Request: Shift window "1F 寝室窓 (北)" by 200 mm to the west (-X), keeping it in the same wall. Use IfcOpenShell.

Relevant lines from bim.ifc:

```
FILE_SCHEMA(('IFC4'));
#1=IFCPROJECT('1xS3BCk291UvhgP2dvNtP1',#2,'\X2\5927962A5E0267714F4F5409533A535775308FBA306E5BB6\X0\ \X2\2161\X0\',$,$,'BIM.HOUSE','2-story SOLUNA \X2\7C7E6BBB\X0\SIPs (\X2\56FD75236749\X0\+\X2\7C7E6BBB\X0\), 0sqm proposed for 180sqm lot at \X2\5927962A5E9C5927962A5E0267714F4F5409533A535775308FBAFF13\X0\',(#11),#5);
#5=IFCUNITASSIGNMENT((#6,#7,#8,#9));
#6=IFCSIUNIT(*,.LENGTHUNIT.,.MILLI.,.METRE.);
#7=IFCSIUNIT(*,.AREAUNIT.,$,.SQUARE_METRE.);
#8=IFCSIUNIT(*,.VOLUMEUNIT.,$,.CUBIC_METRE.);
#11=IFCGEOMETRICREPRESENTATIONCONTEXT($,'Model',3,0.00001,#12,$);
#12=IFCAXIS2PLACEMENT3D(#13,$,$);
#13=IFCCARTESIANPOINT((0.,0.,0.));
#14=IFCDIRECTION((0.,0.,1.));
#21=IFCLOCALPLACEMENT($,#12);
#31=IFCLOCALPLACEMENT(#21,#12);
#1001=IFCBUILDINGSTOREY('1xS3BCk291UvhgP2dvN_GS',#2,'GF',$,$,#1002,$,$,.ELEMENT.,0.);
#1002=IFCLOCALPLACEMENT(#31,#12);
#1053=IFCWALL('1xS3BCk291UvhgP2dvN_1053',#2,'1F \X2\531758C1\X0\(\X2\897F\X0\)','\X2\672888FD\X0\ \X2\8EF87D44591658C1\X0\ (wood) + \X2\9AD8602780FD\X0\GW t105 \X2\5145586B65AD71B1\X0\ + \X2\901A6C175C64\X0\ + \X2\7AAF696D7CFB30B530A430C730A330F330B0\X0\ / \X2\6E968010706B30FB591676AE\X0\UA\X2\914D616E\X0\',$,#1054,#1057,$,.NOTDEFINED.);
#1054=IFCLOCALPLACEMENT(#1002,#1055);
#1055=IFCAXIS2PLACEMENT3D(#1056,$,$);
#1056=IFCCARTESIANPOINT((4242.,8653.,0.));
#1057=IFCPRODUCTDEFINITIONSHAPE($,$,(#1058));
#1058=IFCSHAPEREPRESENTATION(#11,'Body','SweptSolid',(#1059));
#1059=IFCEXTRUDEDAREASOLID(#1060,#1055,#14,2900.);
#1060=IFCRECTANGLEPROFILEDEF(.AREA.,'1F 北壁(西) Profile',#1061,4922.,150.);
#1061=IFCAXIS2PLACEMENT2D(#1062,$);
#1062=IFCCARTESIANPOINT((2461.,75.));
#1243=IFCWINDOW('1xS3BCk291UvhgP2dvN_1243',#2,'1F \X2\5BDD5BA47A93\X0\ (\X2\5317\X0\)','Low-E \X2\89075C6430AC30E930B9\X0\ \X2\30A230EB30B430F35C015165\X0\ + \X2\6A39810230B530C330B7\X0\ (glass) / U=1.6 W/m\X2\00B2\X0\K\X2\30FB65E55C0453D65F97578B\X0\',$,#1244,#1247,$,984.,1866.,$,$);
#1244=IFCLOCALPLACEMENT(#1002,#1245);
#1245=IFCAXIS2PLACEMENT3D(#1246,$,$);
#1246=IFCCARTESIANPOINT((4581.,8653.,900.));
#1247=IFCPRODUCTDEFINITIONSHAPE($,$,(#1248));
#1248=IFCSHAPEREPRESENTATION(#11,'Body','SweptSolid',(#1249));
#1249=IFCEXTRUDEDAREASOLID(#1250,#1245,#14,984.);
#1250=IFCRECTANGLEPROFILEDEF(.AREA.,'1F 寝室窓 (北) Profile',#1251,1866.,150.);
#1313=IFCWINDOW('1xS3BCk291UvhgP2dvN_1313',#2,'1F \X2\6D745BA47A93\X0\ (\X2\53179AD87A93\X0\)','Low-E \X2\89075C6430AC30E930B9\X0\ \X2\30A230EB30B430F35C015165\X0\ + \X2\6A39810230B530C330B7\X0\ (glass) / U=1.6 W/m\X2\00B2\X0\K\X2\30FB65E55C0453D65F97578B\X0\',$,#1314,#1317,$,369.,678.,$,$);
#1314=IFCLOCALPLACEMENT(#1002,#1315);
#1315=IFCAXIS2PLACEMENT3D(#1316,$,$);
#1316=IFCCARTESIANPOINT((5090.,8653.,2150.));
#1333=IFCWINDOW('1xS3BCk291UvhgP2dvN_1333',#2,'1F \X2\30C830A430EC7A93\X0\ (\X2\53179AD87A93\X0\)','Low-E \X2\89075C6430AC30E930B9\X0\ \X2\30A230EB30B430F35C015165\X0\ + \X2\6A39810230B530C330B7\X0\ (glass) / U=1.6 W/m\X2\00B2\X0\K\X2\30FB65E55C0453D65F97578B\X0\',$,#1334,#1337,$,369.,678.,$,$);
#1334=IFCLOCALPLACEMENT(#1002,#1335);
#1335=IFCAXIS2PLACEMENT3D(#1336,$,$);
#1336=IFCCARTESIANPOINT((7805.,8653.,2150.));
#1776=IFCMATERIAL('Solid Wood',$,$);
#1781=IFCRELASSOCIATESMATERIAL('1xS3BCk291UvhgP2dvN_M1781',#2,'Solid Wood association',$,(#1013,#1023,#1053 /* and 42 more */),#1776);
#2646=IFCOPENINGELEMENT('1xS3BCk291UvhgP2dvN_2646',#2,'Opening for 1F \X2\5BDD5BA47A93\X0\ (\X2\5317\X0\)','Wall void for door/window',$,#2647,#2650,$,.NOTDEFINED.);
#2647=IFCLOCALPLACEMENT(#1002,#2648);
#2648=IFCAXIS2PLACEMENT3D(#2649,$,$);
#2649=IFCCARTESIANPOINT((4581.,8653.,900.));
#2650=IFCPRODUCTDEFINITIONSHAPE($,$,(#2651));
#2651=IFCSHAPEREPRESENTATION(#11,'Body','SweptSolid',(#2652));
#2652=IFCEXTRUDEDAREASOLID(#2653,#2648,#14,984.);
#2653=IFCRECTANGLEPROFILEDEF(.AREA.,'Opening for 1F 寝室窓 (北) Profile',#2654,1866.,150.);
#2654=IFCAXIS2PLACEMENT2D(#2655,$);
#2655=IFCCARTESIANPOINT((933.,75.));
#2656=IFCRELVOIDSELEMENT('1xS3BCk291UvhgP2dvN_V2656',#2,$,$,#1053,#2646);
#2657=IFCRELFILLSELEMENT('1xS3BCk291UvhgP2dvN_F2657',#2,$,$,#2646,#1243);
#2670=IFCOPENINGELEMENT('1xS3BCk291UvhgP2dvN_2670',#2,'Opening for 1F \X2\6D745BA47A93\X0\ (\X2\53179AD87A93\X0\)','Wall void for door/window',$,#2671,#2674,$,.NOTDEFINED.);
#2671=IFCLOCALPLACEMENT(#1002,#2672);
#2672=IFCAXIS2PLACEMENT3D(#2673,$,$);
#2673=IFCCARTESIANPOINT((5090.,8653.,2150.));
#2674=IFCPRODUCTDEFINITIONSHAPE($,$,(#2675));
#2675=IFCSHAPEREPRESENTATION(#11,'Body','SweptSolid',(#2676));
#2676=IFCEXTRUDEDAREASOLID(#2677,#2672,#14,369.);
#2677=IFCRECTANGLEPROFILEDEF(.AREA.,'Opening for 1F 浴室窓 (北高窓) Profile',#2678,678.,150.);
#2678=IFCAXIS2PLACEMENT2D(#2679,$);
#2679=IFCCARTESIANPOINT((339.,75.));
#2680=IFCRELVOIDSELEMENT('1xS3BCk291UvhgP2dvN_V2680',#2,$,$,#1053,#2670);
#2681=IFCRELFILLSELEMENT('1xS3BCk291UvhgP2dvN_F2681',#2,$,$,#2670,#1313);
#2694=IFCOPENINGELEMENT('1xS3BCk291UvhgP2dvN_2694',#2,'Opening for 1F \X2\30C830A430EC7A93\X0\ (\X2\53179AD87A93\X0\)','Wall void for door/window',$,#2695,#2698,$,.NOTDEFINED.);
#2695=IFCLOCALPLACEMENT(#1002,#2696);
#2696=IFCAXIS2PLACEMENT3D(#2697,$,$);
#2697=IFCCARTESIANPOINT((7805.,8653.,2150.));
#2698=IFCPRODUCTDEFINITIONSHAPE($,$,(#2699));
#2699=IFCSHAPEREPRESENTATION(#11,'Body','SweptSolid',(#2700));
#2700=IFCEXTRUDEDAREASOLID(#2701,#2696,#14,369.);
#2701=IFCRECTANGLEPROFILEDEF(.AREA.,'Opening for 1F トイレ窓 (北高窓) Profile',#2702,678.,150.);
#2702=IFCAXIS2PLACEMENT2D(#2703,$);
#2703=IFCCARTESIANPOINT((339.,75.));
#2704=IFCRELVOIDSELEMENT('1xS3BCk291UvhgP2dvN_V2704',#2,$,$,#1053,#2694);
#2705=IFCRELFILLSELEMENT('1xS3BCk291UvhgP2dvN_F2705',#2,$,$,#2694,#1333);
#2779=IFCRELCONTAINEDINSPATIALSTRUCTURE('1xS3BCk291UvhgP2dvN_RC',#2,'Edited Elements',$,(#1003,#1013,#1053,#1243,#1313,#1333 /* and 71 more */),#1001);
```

```python
import ifcopenshell
import ifcopenshell.api.geometry
import ifcopenshell.util.placement

model = ifcopenshell.open("bim.ifc")

window = model.by_guid("1xS3BCk291UvhgP2dvN_1243")
opening = window.FillsVoids[0].RelatingOpeningElement
wall = opening.VoidsElements[0].RelatingBuildingElement

wall_matrix = ifcopenshell.util.placement.get_local_placement(wall.ObjectPlacement)
shift = wall_matrix[:3, 0] * -200.0
before = ifcopenshell.util.placement.get_local_placement(window.ObjectPlacement)[:3, 3].copy()

# The window is not placed relative to its opening, so move both.
for product in (opening, window):
    matrix = ifcopenshell.util.placement.get_local_placement(product.ObjectPlacement)
    matrix[:3, 3] += shift
    ifcopenshell.api.geometry.edit_object_placement(model, product=product, matrix=matrix, is_si=False)

after = ifcopenshell.util.placement.get_local_placement(window.ObjectPlacement)[:3, 3]
print("window moved by", (after - before).round(3) + 0.0)

model.write("bim-out.ifc")
```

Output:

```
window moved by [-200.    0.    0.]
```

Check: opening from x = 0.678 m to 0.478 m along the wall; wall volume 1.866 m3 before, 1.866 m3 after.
